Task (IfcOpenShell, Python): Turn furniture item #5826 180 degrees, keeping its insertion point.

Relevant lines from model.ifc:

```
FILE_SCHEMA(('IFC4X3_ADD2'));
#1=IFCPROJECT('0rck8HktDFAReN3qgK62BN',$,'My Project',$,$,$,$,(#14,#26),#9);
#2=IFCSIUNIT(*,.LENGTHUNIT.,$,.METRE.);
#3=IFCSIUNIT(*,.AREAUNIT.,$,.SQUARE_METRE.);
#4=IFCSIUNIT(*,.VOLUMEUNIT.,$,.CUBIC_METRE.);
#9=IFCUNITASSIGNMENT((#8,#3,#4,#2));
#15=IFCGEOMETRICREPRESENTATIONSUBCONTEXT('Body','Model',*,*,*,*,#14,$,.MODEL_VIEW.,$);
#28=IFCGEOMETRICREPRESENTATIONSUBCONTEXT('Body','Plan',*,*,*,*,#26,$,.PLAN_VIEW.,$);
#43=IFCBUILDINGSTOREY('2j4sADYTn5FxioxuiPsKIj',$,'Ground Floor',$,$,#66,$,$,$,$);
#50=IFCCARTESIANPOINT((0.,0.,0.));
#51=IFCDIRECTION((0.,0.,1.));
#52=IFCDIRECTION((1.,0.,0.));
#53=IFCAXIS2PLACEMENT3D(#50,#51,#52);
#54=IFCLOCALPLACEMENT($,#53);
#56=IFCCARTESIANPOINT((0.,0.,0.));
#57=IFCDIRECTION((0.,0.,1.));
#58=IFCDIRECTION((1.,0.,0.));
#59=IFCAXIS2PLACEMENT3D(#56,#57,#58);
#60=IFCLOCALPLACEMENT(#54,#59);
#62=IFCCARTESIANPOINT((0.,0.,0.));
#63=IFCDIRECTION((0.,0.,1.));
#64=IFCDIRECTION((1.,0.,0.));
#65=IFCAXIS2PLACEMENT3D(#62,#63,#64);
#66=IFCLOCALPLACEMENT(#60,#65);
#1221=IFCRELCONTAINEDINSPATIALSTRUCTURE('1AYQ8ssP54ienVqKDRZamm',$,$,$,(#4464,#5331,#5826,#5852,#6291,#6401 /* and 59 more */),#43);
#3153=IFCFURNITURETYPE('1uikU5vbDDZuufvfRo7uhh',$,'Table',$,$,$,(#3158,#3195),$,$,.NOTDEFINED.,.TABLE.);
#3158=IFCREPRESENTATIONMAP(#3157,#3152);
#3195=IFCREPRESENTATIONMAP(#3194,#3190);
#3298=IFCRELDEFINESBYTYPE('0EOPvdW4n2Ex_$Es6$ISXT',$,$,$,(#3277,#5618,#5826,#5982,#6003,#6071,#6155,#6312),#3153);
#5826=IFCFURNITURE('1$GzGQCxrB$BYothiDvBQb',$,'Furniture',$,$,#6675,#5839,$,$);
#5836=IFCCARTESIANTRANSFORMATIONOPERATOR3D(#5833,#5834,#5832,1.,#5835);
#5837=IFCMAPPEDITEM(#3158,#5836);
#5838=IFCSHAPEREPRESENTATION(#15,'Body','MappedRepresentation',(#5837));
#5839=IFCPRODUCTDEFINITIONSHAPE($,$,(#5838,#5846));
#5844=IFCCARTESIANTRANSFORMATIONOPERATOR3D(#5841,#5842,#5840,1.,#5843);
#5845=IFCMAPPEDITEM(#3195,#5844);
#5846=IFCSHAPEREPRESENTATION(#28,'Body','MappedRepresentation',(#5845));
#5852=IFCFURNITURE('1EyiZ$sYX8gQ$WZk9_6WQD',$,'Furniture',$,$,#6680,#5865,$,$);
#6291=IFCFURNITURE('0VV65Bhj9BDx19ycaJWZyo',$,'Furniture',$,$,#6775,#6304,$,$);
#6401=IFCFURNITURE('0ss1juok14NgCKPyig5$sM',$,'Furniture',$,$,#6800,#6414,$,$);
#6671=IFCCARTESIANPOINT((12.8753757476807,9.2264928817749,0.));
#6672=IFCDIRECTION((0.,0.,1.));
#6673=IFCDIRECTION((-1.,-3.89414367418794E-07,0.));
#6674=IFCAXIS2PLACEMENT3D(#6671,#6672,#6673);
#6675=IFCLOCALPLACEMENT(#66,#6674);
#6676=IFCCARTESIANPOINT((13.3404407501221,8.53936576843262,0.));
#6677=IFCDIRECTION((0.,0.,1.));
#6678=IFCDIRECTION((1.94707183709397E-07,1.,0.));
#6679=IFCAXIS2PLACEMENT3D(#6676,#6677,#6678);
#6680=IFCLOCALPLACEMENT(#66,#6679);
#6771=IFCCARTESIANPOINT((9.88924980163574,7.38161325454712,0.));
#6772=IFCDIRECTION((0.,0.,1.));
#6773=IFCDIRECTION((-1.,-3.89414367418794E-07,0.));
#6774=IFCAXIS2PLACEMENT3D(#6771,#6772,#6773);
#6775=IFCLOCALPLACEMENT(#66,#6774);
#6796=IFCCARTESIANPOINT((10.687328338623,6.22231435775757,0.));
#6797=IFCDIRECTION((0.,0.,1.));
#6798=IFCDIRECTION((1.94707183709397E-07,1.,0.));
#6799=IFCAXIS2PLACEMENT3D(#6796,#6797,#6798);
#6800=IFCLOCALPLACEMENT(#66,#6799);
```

```python
import ifcopenshell
import ifcopenshell.api.geometry
import ifcopenshell.util.placement

model = ifcopenshell.open("model.ifc")

item = model.by_guid("1$GzGQCxrB$BYothiDvBQb")
matrix = ifcopenshell.util.placement.get_local_placement(item.ObjectPlacement)
matrix = matrix @ ifcopenshell.util.placement.rotation(180, "Z")
ifcopenshell.api.geometry.edit_object_placement(model, product=item, matrix=matrix, is_si=False)

print(ifcopenshell.util.placement.get_local_placement(item.ObjectPlacement).round(3) + 0.0)

model.write("model_v2.ifc")
```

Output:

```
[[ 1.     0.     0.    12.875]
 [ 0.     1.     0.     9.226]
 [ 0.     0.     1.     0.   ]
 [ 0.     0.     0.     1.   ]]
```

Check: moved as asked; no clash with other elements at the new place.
